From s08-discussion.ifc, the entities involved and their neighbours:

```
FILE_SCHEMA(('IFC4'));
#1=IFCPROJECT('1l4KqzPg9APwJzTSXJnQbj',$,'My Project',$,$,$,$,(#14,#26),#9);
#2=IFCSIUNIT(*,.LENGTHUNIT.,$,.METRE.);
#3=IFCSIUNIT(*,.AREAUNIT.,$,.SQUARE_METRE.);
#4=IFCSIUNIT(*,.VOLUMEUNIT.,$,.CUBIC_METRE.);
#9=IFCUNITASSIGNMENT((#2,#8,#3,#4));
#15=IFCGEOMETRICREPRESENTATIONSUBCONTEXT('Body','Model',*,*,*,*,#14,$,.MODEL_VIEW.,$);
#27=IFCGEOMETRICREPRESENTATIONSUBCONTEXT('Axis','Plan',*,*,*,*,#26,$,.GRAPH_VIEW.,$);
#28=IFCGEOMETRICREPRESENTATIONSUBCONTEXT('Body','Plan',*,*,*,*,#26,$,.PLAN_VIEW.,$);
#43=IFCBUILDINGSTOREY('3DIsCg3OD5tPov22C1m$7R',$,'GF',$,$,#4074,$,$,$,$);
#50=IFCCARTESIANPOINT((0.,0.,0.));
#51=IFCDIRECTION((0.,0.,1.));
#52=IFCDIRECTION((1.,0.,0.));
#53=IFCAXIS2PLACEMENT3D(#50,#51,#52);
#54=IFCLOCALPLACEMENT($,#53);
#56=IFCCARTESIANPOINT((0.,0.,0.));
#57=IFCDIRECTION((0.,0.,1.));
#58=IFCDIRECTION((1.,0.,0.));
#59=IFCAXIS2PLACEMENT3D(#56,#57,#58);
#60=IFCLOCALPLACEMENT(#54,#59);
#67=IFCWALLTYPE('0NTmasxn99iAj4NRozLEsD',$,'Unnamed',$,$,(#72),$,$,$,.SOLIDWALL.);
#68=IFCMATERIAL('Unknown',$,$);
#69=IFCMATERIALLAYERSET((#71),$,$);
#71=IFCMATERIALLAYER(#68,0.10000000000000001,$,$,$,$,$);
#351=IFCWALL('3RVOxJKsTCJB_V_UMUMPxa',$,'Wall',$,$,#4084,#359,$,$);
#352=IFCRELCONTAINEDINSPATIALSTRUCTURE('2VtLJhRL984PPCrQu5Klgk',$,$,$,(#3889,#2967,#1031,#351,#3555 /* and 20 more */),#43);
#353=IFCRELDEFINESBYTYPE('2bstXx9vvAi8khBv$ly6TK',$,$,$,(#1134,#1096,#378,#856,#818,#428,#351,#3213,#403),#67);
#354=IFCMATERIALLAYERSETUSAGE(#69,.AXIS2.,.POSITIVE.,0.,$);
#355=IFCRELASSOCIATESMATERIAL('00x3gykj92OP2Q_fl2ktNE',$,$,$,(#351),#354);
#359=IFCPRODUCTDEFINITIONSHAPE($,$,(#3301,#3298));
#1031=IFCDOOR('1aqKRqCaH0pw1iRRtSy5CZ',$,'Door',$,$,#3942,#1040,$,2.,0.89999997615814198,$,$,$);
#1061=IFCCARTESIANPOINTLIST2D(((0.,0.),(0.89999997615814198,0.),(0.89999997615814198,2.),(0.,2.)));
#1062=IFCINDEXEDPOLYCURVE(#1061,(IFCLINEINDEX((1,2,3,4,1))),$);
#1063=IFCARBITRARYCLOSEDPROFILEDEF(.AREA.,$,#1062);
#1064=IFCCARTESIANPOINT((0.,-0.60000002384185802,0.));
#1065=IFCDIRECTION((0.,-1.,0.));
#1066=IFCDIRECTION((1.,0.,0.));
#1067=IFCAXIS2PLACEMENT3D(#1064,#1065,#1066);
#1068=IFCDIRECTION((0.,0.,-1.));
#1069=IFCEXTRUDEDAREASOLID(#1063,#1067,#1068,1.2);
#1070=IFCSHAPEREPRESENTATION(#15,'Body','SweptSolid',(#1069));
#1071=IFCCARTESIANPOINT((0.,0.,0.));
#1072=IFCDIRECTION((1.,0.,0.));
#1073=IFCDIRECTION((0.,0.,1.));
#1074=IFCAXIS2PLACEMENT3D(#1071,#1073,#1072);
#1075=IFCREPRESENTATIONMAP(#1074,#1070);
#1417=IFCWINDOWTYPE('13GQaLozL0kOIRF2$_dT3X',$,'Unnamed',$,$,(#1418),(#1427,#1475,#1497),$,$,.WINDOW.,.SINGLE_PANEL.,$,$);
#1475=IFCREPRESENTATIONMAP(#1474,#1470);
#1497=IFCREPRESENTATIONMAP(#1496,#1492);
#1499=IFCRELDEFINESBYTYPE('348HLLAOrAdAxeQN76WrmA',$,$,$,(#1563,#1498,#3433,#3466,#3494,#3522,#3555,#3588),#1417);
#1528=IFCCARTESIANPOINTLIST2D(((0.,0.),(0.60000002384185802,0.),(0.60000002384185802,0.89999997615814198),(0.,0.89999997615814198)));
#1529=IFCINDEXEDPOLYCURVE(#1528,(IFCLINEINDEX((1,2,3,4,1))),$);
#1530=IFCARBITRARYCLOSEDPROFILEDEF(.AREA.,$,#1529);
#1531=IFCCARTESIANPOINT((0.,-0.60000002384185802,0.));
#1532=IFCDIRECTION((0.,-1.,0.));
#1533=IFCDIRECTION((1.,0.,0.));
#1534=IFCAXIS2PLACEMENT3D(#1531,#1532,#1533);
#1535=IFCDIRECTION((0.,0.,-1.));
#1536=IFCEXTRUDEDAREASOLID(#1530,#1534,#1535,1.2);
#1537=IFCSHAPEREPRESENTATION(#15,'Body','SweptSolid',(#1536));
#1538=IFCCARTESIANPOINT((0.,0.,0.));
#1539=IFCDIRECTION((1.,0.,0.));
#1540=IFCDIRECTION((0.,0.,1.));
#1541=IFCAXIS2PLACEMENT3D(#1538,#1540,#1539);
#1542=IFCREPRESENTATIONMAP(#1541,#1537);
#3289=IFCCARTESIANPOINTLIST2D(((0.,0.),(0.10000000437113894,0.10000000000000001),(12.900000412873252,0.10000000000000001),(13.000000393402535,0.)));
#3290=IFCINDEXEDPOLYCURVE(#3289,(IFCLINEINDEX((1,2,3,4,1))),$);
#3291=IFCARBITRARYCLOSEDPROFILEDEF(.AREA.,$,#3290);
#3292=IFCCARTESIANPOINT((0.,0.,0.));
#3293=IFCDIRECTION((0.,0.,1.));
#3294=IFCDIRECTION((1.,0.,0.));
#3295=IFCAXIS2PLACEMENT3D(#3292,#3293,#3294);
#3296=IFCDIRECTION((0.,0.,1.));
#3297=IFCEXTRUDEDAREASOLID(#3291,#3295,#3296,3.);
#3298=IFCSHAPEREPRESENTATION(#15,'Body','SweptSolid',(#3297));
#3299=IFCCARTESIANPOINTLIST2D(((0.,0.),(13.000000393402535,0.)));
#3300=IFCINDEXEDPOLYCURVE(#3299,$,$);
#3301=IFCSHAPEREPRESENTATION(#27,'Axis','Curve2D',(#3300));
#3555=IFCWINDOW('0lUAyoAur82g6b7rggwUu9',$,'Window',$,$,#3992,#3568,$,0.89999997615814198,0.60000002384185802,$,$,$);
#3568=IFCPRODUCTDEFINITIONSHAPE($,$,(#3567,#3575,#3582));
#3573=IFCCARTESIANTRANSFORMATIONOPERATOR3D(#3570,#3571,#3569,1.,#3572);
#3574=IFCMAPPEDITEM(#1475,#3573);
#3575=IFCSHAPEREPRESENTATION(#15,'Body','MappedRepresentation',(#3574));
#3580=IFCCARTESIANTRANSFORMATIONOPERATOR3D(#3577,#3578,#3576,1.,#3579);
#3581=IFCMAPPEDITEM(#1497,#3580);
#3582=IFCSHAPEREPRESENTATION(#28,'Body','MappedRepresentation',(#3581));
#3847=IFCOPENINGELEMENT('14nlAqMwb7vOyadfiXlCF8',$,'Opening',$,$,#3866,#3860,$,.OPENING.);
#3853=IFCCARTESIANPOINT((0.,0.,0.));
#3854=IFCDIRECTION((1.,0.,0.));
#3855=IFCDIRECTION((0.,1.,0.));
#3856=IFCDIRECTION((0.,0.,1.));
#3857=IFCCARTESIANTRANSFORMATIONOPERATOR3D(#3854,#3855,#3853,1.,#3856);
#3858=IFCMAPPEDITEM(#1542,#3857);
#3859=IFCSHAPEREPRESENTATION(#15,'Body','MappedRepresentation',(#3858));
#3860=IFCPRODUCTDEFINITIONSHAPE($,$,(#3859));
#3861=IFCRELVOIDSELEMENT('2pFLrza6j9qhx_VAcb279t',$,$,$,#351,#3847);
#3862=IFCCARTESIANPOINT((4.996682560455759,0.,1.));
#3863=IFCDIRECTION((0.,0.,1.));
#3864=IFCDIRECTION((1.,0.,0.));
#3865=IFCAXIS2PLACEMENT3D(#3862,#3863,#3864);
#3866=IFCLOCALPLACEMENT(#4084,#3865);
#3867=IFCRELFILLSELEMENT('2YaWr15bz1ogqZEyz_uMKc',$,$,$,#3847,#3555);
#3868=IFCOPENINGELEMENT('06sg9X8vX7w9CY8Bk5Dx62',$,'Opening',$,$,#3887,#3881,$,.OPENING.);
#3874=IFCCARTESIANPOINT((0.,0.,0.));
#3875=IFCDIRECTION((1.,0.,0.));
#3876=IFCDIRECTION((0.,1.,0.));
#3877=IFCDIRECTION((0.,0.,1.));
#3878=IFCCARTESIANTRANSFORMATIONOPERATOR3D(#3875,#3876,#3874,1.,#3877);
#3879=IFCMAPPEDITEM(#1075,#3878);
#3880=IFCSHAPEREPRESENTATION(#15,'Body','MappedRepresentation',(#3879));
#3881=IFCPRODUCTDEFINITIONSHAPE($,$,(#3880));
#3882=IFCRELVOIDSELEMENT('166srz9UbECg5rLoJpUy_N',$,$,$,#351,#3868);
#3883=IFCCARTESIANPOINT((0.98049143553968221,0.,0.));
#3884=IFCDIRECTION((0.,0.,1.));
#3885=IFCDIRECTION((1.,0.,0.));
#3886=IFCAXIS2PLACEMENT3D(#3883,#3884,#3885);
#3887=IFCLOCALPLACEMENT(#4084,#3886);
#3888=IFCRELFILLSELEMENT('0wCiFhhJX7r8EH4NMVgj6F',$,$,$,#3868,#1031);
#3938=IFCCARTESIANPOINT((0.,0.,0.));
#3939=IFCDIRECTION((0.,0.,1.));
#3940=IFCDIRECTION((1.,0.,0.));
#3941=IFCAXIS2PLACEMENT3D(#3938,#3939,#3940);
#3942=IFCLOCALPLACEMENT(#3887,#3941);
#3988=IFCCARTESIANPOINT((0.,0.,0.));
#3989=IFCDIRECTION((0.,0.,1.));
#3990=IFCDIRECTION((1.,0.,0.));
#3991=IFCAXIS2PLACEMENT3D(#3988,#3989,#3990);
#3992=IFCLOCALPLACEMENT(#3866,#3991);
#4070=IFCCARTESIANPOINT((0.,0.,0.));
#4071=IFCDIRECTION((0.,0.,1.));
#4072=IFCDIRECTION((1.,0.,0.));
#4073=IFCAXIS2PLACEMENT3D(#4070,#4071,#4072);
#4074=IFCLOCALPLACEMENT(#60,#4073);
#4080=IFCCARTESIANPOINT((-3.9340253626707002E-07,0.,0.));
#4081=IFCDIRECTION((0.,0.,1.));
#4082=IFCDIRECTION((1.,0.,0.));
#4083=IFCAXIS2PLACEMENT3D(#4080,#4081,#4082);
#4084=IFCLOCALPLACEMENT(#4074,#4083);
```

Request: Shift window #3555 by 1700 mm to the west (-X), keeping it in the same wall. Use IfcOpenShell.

```python
import ifcopenshell
import ifcopenshell.api.geometry
import ifcopenshell.util.placement
import ifcopenshell.util.unit

model = ifcopenshell.open("s08-discussion.ifc")
unit_scale = ifcopenshell.util.unit.calculate_unit_scale(model)

window = model.by_id(3555)
opening = window.FillsVoids[0].RelatingOpeningElement
wall = opening.VoidsElements[0].RelatingBuildingElement

wall_matrix = ifcopenshell.util.placement.get_local_placement(wall.ObjectPlacement)
shift = wall_matrix[:3, 0] * -1.7 / unit_scale
before = ifcopenshell.util.placement.get_local_placement(window.ObjectPlacement)[:3, 3].copy()

# The window is placed relative to its opening, so it follows when the opening moves.
matrix = ifcopenshell.util.placement.get_local_placement(opening.ObjectPlacement)
matrix[:3, 3] += shift
ifcopenshell.api.geometry.edit_object_placement(
    model, product=opening, matrix=matrix, is_si=False, should_transform_children=True
)

after = ifcopenshell.util.placement.get_local_placement(window.ObjectPlacement)[:3, 3]
print("window moved by", (after - before).round(3) + 0.0)

model.write("s08-discussion_edited.ifc")
```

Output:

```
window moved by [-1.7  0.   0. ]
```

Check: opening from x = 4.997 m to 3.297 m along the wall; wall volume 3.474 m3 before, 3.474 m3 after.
